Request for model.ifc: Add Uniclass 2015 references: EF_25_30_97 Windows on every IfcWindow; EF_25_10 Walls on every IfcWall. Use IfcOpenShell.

First a look at what the model holds.

```python
import ifcopenshell

model = ifcopenshell.open("model.ifc")
print(model.schema)
print("classifications:", [c.Name for c in model.by_type("IfcClassification")])
for ifc_class in ("IfcDoor", "IfcRoof", "IfcStair", "IfcWall", "IfcWindow"):
    print(ifc_class, len(model.by_type(ifc_class)))
```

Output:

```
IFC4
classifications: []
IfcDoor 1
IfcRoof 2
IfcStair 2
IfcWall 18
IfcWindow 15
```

```python
import ifcopenshell
import ifcopenshell.api.classification

model = ifcopenshell.open("model.ifc")

system = ifcopenshell.api.classification.add_classification(model, classification="Uniclass 2015")

codes = {
    "IfcWindow": ("EF_25_30_97", "Windows"),
    "IfcWall": ("EF_25_10", "Walls"),
}
for ifc_class, (code, name) in codes.items():
    products = model.by_type(ifc_class)
    ifcopenshell.api.classification.add_reference(
        model, products=products, classification=system, identification=code, name=name
    )
    print(code, len(products))

model.write("model-out.ifc")
```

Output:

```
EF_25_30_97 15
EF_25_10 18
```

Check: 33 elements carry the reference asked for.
